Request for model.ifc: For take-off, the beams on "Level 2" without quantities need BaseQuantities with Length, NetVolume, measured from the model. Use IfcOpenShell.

First a look at what the model holds.

```python
import ifcopenshell
import ifcopenshell.util.element
import ifcopenshell.util.unit

model = ifcopenshell.open("model.ifc")
print(model.schema)
for unit_type in ("LENGTHUNIT", "AREAUNIT", "VOLUMEUNIT"):
    print(unit_type, ifcopenshell.util.unit.calculate_unit_scale(model, unit_type))
storey = next(s for s in model.by_type("IfcBuildingStorey") if s.Name == "Level 2")
beams = [e for e in ifcopenshell.util.element.get_decomposition(storey) if e.is_a("IfcBeam")]
for e in sorted(beams, key=lambda e: e.id()):
    print(e.id(), e.is_a(), e.Name, list(ifcopenshell.util.element.get_psets(e, qtos_only=True)), sep=" | ")
```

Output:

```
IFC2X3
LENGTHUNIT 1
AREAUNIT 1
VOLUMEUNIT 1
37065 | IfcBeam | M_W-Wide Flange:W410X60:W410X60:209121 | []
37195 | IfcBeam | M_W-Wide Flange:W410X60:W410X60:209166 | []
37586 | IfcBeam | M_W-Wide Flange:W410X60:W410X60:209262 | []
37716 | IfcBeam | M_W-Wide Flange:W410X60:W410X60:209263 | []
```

```python
import ifcopenshell
import ifcopenshell.api.pset
import ifcopenshell.geom
import ifcopenshell.util.element
import ifcopenshell.util.shape
import ifcopenshell.util.unit

model = ifcopenshell.open("model.ifc")
unit_scale = ifcopenshell.util.unit.calculate_unit_scale(model)
volume_scale = ifcopenshell.util.unit.calculate_unit_scale(model, "VOLUMEUNIT")
settings = ifcopenshell.geom.settings()

storey = next(s for s in model.by_type("IfcBuildingStorey") if s.Name == "Level 2")
beams = [e for e in ifcopenshell.util.element.get_decomposition(storey) if e.is_a("IfcBeam")]

for e in sorted(beams, key=lambda e: e.id()):
    if ifcopenshell.util.element.get_psets(e, qtos_only=True, should_inherit=False):
        continue
    # Geometry comes back in metres, in the element's own axes.
    shape = ifcopenshell.geom.create_shape(settings, e)
    values = {
        "Length": ifcopenshell.util.shape.get_max_xyz(shape.geometry) / unit_scale,
        "NetVolume": ifcopenshell.util.shape.get_volume(shape.geometry) / volume_scale,
    }
    qto = ifcopenshell.api.pset.add_qto(model, product=e, name="BaseQuantities")
    ifcopenshell.api.pset.edit_qto(model, qto=qto, properties=values)
    print(e.id(), {k: round(v, 3) for k, v in values.items()})

model.write("model_rev.ifc")
```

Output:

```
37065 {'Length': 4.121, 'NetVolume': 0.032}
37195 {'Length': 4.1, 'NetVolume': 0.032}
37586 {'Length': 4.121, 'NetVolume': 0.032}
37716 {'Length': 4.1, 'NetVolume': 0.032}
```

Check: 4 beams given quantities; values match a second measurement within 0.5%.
